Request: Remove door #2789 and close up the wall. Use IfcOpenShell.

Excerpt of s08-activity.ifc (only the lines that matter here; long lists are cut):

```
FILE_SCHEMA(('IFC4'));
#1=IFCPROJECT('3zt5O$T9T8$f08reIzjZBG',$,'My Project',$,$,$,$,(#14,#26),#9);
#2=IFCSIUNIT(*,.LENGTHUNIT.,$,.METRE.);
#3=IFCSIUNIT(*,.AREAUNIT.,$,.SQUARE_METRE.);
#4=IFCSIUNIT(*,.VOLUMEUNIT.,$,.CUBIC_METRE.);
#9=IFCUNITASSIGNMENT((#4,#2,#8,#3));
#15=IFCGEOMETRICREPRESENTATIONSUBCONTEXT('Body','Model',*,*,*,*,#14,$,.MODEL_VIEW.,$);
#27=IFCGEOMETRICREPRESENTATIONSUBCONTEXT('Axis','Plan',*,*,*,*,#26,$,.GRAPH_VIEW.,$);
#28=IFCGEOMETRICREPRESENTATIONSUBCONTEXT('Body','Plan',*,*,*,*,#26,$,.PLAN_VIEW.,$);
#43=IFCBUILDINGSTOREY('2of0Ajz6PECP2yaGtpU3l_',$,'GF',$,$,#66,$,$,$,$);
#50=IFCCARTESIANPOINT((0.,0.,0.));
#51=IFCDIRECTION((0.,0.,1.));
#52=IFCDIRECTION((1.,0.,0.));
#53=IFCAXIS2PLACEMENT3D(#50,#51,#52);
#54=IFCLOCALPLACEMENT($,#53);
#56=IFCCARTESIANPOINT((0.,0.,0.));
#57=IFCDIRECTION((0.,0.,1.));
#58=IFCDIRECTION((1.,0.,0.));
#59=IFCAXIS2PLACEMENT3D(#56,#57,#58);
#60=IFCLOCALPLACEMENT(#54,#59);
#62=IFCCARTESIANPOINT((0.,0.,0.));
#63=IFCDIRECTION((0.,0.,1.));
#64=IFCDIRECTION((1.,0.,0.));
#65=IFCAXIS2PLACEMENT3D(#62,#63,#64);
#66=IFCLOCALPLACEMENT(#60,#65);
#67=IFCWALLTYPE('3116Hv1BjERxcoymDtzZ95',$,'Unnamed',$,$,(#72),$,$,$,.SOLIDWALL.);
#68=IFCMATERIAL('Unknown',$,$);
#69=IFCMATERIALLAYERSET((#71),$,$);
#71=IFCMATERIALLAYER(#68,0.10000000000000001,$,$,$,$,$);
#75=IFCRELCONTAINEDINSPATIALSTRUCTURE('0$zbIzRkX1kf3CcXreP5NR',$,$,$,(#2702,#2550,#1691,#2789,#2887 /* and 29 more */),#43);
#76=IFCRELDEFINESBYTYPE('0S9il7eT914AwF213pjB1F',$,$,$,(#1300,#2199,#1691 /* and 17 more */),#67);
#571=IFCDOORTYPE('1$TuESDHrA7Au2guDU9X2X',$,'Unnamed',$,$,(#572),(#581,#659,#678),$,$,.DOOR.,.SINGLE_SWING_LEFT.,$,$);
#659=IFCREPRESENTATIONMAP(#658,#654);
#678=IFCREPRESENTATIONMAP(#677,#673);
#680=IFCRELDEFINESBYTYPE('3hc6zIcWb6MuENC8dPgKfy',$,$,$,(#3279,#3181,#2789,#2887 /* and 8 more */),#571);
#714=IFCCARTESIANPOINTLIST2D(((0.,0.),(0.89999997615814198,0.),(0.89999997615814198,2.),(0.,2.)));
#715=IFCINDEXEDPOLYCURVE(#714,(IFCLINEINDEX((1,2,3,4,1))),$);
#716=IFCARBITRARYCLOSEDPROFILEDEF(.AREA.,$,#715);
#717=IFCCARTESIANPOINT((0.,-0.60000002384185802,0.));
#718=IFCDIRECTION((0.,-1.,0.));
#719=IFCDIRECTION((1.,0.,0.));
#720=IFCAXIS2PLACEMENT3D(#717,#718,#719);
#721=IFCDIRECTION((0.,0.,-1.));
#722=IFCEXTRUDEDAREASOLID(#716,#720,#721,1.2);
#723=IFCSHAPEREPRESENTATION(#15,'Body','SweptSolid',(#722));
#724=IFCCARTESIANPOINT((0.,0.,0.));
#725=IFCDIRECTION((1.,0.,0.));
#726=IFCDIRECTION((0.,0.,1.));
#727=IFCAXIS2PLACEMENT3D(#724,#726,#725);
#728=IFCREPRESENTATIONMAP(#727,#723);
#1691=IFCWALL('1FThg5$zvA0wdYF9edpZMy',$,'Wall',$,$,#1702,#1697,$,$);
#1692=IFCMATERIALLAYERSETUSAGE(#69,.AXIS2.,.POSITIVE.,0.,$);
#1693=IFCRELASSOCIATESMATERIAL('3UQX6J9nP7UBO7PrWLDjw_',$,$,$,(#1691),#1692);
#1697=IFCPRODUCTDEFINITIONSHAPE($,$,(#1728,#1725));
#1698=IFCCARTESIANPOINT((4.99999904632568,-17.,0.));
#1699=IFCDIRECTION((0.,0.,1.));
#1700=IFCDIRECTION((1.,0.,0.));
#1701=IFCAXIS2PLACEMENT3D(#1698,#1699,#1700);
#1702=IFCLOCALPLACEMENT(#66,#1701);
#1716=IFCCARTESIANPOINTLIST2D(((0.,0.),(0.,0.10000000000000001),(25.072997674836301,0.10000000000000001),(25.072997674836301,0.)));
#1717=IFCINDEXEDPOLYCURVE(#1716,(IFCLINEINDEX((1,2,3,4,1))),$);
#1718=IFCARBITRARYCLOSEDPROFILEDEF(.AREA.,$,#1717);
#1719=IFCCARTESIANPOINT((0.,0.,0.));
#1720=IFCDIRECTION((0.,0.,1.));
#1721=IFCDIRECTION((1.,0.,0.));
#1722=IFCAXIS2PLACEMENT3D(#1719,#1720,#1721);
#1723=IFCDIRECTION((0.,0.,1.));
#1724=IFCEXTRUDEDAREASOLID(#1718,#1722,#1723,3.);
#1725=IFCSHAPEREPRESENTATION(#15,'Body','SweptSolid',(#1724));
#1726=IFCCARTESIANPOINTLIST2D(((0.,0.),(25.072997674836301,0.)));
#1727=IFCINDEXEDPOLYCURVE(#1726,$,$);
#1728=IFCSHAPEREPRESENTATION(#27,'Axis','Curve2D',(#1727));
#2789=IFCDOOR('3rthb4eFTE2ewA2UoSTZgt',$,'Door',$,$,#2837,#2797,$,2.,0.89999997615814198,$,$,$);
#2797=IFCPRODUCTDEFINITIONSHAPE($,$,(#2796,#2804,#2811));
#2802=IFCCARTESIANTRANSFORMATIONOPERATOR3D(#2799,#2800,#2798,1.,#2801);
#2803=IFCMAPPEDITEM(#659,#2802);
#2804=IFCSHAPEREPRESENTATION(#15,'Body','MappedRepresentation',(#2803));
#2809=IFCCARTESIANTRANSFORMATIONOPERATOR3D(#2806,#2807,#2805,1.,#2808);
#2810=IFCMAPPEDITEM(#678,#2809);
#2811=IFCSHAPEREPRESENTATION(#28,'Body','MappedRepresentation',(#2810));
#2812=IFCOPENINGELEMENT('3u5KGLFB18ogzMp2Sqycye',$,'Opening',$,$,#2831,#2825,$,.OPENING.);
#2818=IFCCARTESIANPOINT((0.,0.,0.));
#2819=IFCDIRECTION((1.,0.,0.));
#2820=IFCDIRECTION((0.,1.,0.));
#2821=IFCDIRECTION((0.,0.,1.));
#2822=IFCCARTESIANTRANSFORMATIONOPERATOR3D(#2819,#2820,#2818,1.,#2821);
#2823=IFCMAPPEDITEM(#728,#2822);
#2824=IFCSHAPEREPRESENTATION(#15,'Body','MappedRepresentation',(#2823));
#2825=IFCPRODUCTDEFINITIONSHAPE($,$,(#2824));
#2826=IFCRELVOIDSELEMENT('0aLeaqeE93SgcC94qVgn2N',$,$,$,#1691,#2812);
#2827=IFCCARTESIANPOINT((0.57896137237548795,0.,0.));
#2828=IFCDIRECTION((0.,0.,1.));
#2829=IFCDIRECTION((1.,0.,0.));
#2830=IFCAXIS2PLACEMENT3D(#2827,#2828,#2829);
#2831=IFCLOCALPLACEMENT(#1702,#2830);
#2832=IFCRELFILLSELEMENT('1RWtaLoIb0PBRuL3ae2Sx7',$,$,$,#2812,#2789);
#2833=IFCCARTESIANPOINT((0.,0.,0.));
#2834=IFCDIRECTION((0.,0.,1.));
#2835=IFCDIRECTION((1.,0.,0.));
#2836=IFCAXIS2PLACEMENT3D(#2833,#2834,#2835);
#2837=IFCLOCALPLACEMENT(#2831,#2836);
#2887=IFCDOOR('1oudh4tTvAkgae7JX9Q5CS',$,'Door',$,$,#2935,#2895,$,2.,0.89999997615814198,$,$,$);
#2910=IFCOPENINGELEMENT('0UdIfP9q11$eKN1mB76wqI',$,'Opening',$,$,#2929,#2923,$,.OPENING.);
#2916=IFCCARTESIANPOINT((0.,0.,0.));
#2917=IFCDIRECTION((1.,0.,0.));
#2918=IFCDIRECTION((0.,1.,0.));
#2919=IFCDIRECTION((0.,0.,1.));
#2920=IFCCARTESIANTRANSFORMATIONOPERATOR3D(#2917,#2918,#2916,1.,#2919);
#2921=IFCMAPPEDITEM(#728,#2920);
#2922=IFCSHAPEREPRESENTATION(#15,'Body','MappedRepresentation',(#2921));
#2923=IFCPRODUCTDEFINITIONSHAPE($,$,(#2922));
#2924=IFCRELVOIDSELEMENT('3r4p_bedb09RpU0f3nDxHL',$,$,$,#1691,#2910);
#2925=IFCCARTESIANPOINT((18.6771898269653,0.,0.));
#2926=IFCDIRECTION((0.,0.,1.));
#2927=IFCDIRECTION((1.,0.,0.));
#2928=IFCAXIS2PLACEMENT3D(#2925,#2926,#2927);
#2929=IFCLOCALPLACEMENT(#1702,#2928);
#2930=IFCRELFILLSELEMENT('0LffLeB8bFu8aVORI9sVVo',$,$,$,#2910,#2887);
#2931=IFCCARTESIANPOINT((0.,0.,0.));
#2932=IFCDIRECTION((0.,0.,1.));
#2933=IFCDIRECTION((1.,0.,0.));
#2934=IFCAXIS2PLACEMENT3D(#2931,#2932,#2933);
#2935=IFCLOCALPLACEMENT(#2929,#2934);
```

```python
import ifcopenshell
import ifcopenshell.api.feature
import ifcopenshell.api.root
import ifcopenshell.geom
import ifcopenshell.util.shape

model = ifcopenshell.open("s08-activity.ifc")
settings = ifcopenshell.geom.settings()


def volume(element):
    """Net volume in cubic metres, openings subtracted."""
    shape = ifcopenshell.geom.create_shape(settings, element)
    return ifcopenshell.util.shape.get_volume(shape.geometry)


door = model.by_guid("3rthb4eFTE2ewA2UoSTZgt")
opening = door.FillsVoids[0].RelatingOpeningElement
wall = opening.VoidsElements[0].RelatingBuildingElement
before = volume(wall)

ifcopenshell.api.root.remove_product(model, product=door)
ifcopenshell.api.feature.remove_feature(model, feature=opening)

after = volume(wall)

print(f"wall volume {before:.3f} -> {after:.3f} m3")

model.write("s08-activity-out.ifc")
```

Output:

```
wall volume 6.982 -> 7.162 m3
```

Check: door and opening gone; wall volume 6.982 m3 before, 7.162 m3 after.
